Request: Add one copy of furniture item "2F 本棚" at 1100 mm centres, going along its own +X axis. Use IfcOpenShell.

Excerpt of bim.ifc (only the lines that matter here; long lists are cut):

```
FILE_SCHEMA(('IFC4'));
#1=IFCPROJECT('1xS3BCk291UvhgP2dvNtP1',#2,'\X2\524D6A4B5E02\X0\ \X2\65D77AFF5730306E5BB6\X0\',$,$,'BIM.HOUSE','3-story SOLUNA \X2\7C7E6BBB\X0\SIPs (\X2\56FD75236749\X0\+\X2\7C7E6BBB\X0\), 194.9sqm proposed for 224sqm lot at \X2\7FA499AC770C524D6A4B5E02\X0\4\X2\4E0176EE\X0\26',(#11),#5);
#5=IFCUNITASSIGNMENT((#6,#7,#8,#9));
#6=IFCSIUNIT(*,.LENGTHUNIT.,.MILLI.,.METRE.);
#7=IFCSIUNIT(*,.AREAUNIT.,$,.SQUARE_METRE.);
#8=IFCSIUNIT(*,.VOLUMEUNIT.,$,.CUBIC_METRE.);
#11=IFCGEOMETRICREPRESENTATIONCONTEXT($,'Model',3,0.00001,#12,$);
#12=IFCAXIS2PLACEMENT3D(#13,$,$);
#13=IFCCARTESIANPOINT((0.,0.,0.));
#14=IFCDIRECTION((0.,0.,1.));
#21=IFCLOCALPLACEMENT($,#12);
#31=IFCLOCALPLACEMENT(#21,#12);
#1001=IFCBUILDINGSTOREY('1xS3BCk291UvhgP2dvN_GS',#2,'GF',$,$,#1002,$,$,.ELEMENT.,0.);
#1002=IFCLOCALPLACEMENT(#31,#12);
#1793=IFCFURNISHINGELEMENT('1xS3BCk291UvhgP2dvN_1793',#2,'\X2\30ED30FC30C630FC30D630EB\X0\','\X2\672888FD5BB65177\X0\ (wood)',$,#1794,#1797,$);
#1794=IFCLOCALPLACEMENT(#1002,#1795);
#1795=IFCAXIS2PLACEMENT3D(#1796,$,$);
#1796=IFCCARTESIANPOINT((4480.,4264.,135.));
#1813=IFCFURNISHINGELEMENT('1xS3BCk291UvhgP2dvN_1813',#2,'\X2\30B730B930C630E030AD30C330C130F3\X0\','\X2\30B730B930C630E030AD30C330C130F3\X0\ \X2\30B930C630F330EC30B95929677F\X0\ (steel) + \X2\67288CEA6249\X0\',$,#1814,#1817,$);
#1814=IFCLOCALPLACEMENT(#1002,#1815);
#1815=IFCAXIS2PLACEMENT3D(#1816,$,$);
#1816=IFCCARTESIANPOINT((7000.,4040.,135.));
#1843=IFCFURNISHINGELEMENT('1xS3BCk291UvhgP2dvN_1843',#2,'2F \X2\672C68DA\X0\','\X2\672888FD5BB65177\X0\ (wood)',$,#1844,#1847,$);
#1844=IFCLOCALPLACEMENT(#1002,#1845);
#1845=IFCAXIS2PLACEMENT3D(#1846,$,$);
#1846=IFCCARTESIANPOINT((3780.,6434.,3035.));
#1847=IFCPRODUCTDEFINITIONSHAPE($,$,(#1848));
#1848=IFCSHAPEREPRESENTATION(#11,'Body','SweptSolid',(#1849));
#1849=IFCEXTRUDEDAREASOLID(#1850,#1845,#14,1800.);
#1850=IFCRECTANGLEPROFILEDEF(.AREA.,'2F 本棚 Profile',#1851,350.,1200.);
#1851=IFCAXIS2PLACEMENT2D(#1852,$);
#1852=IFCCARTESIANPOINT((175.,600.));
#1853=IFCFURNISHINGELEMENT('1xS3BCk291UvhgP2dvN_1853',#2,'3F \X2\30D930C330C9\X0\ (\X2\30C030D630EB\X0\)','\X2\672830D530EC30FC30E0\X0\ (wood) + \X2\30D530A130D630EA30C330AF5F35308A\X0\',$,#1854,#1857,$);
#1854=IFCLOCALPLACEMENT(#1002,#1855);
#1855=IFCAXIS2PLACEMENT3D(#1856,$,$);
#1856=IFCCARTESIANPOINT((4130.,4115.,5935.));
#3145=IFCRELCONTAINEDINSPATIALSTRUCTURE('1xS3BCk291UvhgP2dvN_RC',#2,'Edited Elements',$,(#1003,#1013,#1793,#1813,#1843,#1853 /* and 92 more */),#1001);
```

```python
import ifcopenshell
import ifcopenshell.api.geometry
import ifcopenshell.api.root
import ifcopenshell.util.element
import ifcopenshell.util.placement

model = ifcopenshell.open("bim.ifc")


def reuse_history(source, copy):
    """copy_class also copies each property set's owner history, people and application; keep the originals."""
    for rel in copy.IsDefinedBy:
        if rel.is_a("IfcRelDefinesByProperties") and (history := rel.RelatingPropertyDefinition.OwnerHistory):
            rel.RelatingPropertyDefinition.OwnerHistory = source.OwnerHistory
            ifcopenshell.util.element.remove_deep2(model, history)


source = model.by_id(1843)
base = ifcopenshell.util.placement.get_local_placement(source.ObjectPlacement)
step = base[:3, 0] * 1100.0

for i in range(1, 2):
    copy = ifcopenshell.api.root.copy_class(model, product=source)
    copy.Representation = ifcopenshell.util.element.copy_deep(
        model, source.Representation, exclude=["IfcGeometricRepresentationContext", "IfcRepresentationMap"]
    )
    reuse_history(source, copy)
    matrix = base.copy()
    matrix[:3, 3] += i * step
    print("added at", matrix[:3, 3].round(3) + 0.0)
    ifcopenshell.api.geometry.edit_object_placement(model, product=copy, matrix=matrix, is_si=False)

model.write("bim-out.ifc")
```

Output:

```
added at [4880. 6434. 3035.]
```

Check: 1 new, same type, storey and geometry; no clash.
